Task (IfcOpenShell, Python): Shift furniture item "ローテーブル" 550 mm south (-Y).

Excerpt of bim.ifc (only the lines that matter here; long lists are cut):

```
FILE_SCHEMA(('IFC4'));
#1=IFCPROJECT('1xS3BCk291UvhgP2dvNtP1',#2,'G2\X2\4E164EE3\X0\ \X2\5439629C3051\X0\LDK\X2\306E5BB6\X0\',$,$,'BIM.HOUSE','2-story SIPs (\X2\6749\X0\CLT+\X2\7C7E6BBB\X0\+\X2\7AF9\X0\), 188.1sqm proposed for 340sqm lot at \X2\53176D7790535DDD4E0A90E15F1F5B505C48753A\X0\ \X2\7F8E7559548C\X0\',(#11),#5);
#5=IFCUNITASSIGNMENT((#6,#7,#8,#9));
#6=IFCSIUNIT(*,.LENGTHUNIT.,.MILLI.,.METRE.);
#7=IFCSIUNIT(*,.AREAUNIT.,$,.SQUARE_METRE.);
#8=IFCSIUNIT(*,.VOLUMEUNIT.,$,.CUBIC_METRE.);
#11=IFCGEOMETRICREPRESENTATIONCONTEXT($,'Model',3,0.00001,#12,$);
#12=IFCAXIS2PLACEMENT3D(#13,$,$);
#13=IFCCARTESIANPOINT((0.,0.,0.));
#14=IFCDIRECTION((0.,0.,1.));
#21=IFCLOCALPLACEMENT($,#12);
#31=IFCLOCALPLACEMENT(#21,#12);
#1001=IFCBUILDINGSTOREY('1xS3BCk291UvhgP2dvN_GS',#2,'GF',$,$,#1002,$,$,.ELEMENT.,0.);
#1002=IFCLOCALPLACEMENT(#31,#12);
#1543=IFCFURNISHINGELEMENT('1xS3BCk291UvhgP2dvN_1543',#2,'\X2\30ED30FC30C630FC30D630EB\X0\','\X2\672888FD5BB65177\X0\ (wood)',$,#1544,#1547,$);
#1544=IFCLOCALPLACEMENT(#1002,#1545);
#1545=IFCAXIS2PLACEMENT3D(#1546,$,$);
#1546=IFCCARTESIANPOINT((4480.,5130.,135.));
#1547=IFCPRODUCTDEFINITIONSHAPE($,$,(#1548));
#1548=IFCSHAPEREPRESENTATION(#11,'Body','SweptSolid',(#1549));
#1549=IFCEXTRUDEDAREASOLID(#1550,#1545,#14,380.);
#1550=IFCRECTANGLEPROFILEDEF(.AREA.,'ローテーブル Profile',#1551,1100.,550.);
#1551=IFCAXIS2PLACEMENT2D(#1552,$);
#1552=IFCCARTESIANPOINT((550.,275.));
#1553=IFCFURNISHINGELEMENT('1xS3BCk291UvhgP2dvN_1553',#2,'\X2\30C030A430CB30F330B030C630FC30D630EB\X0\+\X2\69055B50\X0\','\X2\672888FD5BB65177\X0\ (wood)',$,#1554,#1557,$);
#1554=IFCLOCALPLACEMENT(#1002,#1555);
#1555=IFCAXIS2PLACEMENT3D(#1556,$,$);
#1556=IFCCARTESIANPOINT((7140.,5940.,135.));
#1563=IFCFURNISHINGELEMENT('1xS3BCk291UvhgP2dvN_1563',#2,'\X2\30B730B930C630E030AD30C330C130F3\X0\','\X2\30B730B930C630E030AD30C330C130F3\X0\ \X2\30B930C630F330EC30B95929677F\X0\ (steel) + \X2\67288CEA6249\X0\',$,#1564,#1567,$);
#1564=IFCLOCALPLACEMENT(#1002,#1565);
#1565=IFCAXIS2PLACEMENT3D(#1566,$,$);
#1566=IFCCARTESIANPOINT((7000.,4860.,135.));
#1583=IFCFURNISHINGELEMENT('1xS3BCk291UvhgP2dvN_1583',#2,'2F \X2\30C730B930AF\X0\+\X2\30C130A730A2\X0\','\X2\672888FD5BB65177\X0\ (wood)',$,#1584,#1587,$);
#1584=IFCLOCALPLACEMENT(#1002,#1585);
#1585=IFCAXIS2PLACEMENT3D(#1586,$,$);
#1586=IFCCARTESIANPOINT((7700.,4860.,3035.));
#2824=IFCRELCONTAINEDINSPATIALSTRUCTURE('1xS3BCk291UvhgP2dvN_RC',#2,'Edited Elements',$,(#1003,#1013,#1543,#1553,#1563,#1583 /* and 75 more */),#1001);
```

```python
import ifcopenshell
import ifcopenshell.api.geometry
import ifcopenshell.util.placement
import ifcopenshell.util.unit

model = ifcopenshell.open("bim.ifc")
unit_scale = ifcopenshell.util.unit.calculate_unit_scale(model)

item = model.by_guid("1xS3BCk291UvhgP2dvN_1543")
matrix = ifcopenshell.util.placement.get_local_placement(item.ObjectPlacement)
matrix[1, 3] -= 0.55 / unit_scale
ifcopenshell.api.geometry.edit_object_placement(model, product=item, matrix=matrix, is_si=False)

print(ifcopenshell.util.placement.get_local_placement(item.ObjectPlacement).round(3) + 0.0)

model.write("bim_rev.ifc")
```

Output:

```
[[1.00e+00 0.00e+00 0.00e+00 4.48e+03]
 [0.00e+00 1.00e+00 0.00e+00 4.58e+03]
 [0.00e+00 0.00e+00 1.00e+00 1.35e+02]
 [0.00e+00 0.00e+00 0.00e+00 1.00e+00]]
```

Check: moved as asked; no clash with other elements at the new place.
